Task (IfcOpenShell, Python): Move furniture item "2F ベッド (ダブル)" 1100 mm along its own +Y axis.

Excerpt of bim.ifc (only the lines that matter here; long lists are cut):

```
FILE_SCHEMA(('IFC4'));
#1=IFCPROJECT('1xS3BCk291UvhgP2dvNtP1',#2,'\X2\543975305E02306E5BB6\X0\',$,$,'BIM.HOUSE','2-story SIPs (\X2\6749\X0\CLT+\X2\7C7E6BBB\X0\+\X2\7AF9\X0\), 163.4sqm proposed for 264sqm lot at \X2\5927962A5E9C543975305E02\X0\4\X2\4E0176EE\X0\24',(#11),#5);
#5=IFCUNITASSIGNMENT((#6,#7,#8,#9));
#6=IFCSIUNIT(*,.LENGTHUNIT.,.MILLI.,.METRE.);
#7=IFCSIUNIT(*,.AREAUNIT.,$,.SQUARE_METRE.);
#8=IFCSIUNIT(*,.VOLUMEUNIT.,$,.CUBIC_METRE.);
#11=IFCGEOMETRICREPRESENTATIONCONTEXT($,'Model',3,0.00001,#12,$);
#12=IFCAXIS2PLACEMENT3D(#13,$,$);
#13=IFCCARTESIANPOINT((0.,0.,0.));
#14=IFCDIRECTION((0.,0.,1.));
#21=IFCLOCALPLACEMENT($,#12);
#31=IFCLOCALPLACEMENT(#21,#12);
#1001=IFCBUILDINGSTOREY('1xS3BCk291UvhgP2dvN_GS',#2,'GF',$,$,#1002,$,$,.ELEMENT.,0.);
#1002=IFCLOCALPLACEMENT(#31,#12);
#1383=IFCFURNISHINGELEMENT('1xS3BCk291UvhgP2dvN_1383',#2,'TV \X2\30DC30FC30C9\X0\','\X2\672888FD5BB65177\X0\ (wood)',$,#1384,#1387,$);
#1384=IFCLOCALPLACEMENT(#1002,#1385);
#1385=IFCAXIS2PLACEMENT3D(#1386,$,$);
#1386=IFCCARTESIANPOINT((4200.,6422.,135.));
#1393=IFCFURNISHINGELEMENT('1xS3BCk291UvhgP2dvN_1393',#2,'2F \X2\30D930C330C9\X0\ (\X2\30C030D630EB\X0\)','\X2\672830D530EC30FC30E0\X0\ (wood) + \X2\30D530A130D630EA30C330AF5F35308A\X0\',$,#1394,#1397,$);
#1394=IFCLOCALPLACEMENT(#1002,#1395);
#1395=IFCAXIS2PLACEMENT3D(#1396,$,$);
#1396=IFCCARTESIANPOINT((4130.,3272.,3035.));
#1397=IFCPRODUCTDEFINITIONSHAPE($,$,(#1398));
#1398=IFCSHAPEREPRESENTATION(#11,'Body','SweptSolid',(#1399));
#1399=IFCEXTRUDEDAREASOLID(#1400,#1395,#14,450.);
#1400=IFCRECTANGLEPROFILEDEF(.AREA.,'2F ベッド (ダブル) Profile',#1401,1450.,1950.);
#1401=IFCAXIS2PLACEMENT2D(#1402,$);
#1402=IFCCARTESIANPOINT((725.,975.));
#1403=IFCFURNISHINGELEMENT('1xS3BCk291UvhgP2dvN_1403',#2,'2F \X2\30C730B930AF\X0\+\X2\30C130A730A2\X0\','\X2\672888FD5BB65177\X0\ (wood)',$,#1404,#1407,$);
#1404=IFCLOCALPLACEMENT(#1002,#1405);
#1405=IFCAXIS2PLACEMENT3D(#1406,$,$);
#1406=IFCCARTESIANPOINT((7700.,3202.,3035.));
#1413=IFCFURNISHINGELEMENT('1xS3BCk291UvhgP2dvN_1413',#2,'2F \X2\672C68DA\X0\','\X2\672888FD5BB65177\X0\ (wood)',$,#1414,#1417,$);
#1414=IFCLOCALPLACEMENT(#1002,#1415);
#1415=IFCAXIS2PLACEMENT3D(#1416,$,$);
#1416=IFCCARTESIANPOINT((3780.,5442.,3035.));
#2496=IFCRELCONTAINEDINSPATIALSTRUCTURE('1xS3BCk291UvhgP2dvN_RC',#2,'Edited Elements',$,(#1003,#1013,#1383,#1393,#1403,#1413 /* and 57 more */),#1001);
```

```python
import ifcopenshell
import ifcopenshell.api.geometry
import ifcopenshell.util.placement

model = ifcopenshell.open("bim.ifc")

item = model.by_guid("1xS3BCk291UvhgP2dvN_1393")
matrix = ifcopenshell.util.placement.get_local_placement(item.ObjectPlacement)
matrix[:3, 3] += matrix[:3, 1] * 1100.0
ifcopenshell.api.geometry.edit_object_placement(model, product=item, matrix=matrix, is_si=False)

print(ifcopenshell.util.placement.get_local_placement(item.ObjectPlacement).round(3) + 0.0)

model.write("bim_updated.ifc")
```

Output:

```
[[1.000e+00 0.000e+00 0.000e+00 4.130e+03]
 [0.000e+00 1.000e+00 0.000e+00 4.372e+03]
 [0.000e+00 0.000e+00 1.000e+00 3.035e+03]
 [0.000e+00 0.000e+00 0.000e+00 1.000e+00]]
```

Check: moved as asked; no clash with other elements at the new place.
